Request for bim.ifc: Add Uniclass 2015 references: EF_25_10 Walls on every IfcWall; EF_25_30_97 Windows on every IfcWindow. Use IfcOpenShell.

First a look at what the model holds.

```python
import ifcopenshell

model = ifcopenshell.open("bim.ifc")
print(model.schema)
print("classifications:", [c.Name for c in model.by_type("IfcClassification")])
for ifc_class in ("IfcDoor", "IfcRoof", "IfcStair", "IfcWall", "IfcWindow"):
    print(ifc_class, len(model.by_type(ifc_class)))
```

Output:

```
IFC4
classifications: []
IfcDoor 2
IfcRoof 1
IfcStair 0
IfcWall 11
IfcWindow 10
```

```python
import ifcopenshell
import ifcopenshell.api.classification

model = ifcopenshell.open("bim.ifc")

system = ifcopenshell.api.classification.add_classification(model, classification="Uniclass 2015")

codes = {
    "IfcWall": ("EF_25_10", "Walls"),
    "IfcWindow": ("EF_25_30_97", "Windows"),
}
for ifc_class, (code, name) in codes.items():
    products = model.by_type(ifc_class)
    ifcopenshell.api.classification.add_reference(
        model, products=products, classification=system, identification=code, name=name
    )
    print(code, len(products))

model.write("bim_edited.ifc")
```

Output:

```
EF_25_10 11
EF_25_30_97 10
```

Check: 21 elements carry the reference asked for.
